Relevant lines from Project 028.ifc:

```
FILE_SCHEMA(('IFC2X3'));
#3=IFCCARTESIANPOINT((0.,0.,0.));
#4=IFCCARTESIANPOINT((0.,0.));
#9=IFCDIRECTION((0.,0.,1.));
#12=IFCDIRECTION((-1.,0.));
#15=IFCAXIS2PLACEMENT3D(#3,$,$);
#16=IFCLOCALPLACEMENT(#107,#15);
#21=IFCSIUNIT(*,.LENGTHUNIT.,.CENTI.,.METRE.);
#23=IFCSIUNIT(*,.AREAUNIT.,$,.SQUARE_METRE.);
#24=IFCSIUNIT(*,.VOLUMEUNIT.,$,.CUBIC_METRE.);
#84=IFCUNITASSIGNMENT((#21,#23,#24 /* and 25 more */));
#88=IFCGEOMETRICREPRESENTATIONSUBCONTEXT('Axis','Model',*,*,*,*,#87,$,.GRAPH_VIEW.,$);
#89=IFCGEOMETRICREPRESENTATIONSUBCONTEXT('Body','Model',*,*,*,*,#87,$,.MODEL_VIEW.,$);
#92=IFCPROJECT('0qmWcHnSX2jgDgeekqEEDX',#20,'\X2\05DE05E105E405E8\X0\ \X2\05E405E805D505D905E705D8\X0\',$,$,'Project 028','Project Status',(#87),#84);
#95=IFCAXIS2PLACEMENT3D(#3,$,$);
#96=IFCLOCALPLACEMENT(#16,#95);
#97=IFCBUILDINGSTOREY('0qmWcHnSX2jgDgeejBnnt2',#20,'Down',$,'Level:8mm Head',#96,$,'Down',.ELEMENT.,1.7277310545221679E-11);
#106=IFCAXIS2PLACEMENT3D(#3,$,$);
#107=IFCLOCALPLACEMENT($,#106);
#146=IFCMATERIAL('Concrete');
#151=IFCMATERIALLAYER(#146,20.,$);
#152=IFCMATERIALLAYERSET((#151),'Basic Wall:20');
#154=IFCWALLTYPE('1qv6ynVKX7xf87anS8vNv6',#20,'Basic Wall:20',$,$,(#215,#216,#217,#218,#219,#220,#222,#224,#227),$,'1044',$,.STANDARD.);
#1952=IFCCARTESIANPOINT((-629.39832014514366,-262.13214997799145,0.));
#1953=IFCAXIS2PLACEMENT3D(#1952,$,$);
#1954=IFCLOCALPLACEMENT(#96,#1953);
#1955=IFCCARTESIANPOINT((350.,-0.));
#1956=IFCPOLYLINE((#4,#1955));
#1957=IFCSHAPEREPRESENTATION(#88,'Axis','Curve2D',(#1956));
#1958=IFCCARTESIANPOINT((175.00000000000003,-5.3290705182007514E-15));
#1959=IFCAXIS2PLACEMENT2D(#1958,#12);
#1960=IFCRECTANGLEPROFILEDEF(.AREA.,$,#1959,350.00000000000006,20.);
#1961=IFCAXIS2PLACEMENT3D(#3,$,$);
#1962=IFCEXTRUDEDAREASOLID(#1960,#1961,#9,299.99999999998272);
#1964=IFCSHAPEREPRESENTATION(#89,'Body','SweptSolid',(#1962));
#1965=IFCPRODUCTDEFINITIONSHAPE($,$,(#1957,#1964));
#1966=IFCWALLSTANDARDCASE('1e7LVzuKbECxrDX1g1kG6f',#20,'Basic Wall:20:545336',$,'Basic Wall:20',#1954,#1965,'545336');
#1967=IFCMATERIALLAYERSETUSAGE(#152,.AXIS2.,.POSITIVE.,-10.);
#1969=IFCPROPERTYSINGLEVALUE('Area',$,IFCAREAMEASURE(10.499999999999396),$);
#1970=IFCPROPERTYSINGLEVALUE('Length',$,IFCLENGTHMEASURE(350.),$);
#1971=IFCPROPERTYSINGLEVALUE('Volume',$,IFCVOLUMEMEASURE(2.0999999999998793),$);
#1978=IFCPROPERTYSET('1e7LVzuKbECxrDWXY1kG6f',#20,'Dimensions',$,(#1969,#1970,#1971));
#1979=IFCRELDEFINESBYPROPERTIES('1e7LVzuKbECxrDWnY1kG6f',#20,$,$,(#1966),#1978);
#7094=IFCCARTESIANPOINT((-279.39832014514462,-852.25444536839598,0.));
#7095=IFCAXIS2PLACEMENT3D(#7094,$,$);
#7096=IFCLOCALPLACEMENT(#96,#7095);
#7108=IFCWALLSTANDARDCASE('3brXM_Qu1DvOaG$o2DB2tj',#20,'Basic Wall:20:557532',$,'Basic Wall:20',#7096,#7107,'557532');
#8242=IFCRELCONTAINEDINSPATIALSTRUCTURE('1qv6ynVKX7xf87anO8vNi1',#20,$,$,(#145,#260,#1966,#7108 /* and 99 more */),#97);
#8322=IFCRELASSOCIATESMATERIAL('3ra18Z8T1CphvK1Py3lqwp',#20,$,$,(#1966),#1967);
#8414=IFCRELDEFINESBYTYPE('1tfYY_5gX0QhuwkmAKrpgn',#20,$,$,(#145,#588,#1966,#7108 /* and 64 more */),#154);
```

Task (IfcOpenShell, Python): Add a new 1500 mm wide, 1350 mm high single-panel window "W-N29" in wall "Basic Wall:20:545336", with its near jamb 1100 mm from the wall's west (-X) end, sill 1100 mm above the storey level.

```python
import numpy as np
import ifcopenshell
import ifcopenshell.api.feature
import ifcopenshell.api.geometry
import ifcopenshell.api.pset
import ifcopenshell.api.root
import ifcopenshell.api.spatial
import ifcopenshell.api.type
import ifcopenshell.geom
import ifcopenshell.util.element
import ifcopenshell.util.placement
import ifcopenshell.util.representation
import ifcopenshell.util.shape
import ifcopenshell.util.unit

model = ifcopenshell.open("Project 028.ifc")
unit_scale = ifcopenshell.util.unit.calculate_unit_scale(model)
area_scale = ifcopenshell.util.unit.calculate_unit_scale(model, "AREAUNIT")
volume_scale = ifcopenshell.util.unit.calculate_unit_scale(model, "VOLUMEUNIT")
settings = ifcopenshell.geom.settings()


def volume(element):
    """Net volume in cubic metres, openings subtracted."""
    shape = ifcopenshell.geom.create_shape(settings, element)
    return ifcopenshell.util.shape.get_volume(shape.geometry)


wall = model.by_id(1966)
storey = ifcopenshell.util.element.get_container(wall, ifc_class="IfcBuildingStorey")
context = ifcopenshell.util.representation.get_context(model, "Model", "Body", "MODEL_VIEW")
before = volume(wall)

width, height, from_end, sill = 1.5, 1.35, 1.1, 1.1  # metres

# The wall runs along its own X axis, and the end named is its -X end.
wall_shape = ifcopenshell.geom.create_shape(settings, wall)
x, y, z = ifcopenshell.util.shape.get_vertices(wall_shape.geometry).T
start = x.min() + from_end
face, thickness = float(y.min()), float(y.max() - y.min())
wall_matrix = ifcopenshell.util.placement.get_local_placement(wall.ObjectPlacement)
level = ifcopenshell.util.placement.get_local_placement(storey.ObjectPlacement)[2, 3]


def in_wall(x, y):
    """Placement at x, y metres in the wall's axes, at sill height."""
    matrix = wall_matrix.copy()
    matrix[:, 3] = wall_matrix @ np.array([x / unit_scale, y / unit_scale, 0.0, 1.0])
    matrix[2, 3] = level + sill / unit_scale
    return matrix


# Opening: a box that overshoots both wall faces by 50 mm.
opening = ifcopenshell.api.root.create_entity(model, ifc_class="IfcOpeningElement")
box = ifcopenshell.api.geometry.add_wall_representation(
    model, context=context, length=width, height=height, thickness=thickness + 0.1
)
ifcopenshell.api.geometry.assign_representation(model, product=opening, representation=box)
ifcopenshell.api.geometry.edit_object_placement(model, product=opening, matrix=in_wall(start, face - 0.05), is_si=False)
ifcopenshell.api.feature.add_feature(model, feature=opening, element=wall)

window = ifcopenshell.api.root.create_entity(model, ifc_class="IfcWindow", name="W-N29")
window.OverallWidth, window.OverallHeight = width / unit_scale, height / unit_scale
body = ifcopenshell.api.geometry.add_window_representation(
    model,
    context=context,
    overall_width=window.OverallWidth,
    overall_height=window.OverallHeight,
    partition_type="SINGLE_PANEL",
)
ifcopenshell.api.geometry.assign_representation(model, product=window, representation=body)
ifcopenshell.api.spatial.assign_container(model, products=[window], relating_structure=storey)
fills = ifcopenshell.api.feature.add_filling(model, opening=opening, element=window)
fills.OwnerHistory = window.OwnerHistory  # required in IFC2X3

# IFC2X3 keeps the operation on the window style.
style = ifcopenshell.api.root.create_entity(model, ifc_class="IfcWindowStyle", name="W-N29")
style.OperationType, style.ConstructionType = "SINGLE_PANEL", "NOTDEFINED"
style.ParameterTakesPrecedence = style.Sizeable = False
ifcopenshell.api.type.assign_type(model, related_objects=[window], relating_type=style)

# Centre the window in the wall's thickness.
ifcopenshell.api.geometry.edit_object_placement(model, product=window, matrix=in_wall(start, face), is_si=False)
window_shape = ifcopenshell.geom.create_shape(settings, window)
depth = ifcopenshell.util.shape.get_vertices(window_shape.geometry)[:, 1]
offset = face + thickness / 2 - (depth.min() + depth.max()) / 2
ifcopenshell.api.geometry.edit_object_placement(model, product=window, matrix=in_wall(start, offset), is_si=False)

after = volume(wall)

# Update the wall's stored quantities.
pset = model.by_id(ifcopenshell.util.element.get_pset(wall, "Dimensions", should_inherit=False)["id"])
ifcopenshell.api.pset.edit_pset(model, pset=pset, properties={
    "Area": model.create_entity("IfcAreaMeasure", after / thickness / area_scale),
    "Volume": model.create_entity("IfcVolumeMeasure", after / volume_scale),
})

print(f"wall volume {before:.3f} -> {after:.3f} m3")

model.write("Project 028_rev.ifc")
```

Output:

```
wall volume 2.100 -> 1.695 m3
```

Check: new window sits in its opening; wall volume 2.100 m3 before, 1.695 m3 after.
